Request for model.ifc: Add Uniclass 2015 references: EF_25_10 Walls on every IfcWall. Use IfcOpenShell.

First a look at what the model holds.

```python
import ifcopenshell

model = ifcopenshell.open("model.ifc")
print(model.schema)
print("classifications:", [c.Name for c in model.by_type("IfcClassification")])
for ifc_class in ("IfcDoor", "IfcRoof", "IfcStair", "IfcWall", "IfcWindow"):
    print(ifc_class, len(model.by_type(ifc_class)))
```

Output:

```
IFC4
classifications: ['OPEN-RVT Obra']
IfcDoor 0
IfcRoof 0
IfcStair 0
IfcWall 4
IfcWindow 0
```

```python
import ifcopenshell
import ifcopenshell.api.classification

model = ifcopenshell.open("model.ifc")

system = ifcopenshell.api.classification.add_classification(model, classification="Uniclass 2015")

codes = {
    "IfcWall": ("EF_25_10", "Walls"),
}
for ifc_class, (code, name) in codes.items():
    products = model.by_type(ifc_class)
    ifcopenshell.api.classification.add_reference(
        model, products=products, classification=system, identification=code, name=name
    )
    print(code, len(products))

model.write("model_edited.ifc")
```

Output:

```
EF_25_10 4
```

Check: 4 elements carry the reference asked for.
